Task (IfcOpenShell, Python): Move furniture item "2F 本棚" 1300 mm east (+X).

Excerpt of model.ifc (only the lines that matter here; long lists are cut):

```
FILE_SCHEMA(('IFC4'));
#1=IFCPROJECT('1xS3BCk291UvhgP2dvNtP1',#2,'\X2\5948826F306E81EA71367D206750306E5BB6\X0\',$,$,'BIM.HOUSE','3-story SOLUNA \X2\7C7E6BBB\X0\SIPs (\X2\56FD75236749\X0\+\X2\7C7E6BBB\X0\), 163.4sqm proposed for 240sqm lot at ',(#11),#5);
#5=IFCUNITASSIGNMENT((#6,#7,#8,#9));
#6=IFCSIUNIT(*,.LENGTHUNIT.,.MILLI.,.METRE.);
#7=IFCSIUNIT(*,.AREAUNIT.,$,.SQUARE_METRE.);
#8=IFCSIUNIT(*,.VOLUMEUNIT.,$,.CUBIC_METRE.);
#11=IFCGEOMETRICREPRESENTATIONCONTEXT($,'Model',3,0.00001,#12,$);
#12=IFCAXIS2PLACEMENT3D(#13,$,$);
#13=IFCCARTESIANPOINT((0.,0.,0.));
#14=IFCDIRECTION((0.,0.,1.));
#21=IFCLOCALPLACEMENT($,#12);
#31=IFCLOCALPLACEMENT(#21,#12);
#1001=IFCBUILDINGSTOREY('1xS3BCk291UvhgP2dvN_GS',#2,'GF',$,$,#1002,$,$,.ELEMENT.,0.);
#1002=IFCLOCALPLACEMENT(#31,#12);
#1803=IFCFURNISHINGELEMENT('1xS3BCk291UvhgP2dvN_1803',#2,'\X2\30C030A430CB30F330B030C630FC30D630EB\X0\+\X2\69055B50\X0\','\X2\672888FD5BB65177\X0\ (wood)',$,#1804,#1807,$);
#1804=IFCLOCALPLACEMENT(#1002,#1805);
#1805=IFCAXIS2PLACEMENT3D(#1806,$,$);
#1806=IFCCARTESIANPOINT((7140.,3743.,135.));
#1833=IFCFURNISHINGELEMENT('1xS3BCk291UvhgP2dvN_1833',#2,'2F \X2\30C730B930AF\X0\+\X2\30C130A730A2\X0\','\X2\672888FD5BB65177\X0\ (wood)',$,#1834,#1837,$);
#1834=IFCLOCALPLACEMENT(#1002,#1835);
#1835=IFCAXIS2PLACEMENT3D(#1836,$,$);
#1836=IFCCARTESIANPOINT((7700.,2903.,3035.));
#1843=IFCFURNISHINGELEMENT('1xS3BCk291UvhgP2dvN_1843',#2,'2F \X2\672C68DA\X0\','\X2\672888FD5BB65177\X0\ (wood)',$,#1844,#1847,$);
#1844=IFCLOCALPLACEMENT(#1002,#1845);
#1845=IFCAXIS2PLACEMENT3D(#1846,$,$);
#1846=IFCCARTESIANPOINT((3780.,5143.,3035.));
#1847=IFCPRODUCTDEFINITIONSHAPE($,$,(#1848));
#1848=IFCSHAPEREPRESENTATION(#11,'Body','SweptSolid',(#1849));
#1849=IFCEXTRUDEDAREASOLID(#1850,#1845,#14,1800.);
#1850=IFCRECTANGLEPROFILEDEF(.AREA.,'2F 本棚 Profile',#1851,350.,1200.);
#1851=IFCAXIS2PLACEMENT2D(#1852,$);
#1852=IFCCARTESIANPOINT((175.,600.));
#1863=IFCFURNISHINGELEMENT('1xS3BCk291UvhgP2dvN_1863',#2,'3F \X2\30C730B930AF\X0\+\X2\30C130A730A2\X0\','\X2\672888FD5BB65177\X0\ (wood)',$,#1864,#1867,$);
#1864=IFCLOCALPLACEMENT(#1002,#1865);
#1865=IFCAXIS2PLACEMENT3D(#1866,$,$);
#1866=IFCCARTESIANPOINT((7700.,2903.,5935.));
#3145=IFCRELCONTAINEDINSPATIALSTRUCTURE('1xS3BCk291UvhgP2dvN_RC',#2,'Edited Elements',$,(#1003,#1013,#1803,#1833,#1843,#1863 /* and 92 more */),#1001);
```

```python
import ifcopenshell
import ifcopenshell.api.geometry
import ifcopenshell.util.placement
import ifcopenshell.util.unit

model = ifcopenshell.open("model.ifc")
unit_scale = ifcopenshell.util.unit.calculate_unit_scale(model)

item = model.by_guid("1xS3BCk291UvhgP2dvN_1843")
matrix = ifcopenshell.util.placement.get_local_placement(item.ObjectPlacement)
matrix[0, 3] += 1.3 / unit_scale
ifcopenshell.api.geometry.edit_object_placement(model, product=item, matrix=matrix, is_si=False)

print(ifcopenshell.util.placement.get_local_placement(item.ObjectPlacement).round(3) + 0.0)

model.write("model_updated.ifc")
```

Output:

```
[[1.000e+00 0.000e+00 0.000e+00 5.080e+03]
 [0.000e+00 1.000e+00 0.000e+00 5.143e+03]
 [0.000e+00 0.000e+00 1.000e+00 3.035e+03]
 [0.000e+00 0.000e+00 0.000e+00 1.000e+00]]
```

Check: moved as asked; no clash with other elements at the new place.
